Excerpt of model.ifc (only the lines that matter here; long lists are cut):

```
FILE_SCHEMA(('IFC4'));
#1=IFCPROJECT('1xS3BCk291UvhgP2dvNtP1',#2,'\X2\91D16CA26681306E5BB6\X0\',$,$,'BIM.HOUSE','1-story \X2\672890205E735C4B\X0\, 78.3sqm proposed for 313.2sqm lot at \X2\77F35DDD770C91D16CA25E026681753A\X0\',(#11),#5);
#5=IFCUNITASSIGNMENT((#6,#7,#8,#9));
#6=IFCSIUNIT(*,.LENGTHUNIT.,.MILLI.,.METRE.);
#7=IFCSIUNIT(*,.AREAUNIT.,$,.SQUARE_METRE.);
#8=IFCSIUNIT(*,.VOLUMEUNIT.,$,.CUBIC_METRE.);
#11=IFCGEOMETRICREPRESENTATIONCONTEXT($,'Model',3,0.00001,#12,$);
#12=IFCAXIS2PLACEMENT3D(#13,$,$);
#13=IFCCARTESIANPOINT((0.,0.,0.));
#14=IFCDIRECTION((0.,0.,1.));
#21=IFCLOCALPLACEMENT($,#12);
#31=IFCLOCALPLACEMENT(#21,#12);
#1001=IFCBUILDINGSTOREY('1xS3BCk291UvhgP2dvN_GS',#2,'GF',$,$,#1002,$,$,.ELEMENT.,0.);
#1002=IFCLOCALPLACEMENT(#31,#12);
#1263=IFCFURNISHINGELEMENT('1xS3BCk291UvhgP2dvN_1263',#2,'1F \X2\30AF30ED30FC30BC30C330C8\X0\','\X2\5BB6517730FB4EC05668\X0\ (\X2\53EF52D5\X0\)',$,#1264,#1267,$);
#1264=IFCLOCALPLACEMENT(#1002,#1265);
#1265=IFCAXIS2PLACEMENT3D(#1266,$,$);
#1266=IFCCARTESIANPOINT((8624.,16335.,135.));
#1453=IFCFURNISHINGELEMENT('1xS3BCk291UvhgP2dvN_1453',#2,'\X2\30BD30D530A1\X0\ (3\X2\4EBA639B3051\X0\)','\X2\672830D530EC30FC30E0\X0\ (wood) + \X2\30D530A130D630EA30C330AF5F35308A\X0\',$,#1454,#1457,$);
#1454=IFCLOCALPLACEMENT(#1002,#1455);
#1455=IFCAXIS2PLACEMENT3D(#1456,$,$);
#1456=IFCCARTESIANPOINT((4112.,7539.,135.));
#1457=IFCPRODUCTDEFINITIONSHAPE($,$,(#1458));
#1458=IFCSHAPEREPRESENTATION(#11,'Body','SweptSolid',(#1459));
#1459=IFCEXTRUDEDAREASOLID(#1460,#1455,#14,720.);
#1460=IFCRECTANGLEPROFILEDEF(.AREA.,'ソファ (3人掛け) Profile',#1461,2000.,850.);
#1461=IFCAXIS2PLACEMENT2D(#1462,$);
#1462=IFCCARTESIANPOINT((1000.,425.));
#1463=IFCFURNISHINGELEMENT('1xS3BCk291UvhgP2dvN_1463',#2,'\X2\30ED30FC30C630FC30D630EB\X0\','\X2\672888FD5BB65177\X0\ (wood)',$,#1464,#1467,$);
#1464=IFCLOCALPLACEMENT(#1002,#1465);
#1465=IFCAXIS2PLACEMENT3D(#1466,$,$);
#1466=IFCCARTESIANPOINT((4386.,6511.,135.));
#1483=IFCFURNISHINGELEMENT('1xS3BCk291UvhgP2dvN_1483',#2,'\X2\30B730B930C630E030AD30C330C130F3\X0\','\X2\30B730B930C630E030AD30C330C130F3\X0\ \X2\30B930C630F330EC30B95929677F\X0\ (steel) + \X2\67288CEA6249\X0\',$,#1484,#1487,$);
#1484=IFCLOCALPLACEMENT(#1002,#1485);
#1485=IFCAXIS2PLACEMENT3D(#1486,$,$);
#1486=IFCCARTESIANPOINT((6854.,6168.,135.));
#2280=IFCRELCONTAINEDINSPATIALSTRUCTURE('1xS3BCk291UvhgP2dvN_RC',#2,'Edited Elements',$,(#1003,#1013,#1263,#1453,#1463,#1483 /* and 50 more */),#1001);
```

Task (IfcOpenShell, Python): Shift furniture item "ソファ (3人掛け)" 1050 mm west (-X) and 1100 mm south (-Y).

```python
import ifcopenshell
import ifcopenshell.api.geometry
import ifcopenshell.util.placement
import ifcopenshell.util.unit

model = ifcopenshell.open("model.ifc")
unit_scale = ifcopenshell.util.unit.calculate_unit_scale(model)

item = model.by_id(1453)
matrix = ifcopenshell.util.placement.get_local_placement(item.ObjectPlacement)
matrix[0, 3] -= 1.05 / unit_scale
matrix[1, 3] -= 1.1 / unit_scale
ifcopenshell.api.geometry.edit_object_placement(model, product=item, matrix=matrix, is_si=False)

print(ifcopenshell.util.placement.get_local_placement(item.ObjectPlacement).round(3) + 0.0)

model.write("model-out.ifc")
```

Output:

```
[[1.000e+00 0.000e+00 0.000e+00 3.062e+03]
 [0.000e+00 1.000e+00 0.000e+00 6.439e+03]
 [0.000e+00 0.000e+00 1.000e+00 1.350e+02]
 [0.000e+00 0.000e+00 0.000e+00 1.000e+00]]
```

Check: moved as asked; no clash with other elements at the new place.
